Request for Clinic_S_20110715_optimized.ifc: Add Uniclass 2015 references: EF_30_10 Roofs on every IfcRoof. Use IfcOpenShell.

First a look at what the model holds.

```python
import ifcopenshell

model = ifcopenshell.open("Clinic_S_20110715_optimized.ifc")
print(model.schema)
print("classifications:", [c.Name for c in model.by_type("IfcClassification")])
for ifc_class in ("IfcDoor", "IfcRoof", "IfcStair", "IfcWall", "IfcWindow"):
    print(ifc_class, len(model.by_type(ifc_class)))
```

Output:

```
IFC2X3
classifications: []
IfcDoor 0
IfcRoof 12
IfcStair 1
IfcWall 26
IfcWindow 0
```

```python
import ifcopenshell
import ifcopenshell.api.classification

model = ifcopenshell.open("Clinic_S_20110715_optimized.ifc")

# IFC2X3 requires Source and Edition and has no link from the project to the system.
system = model.create_entity("IfcClassification", Source="NBS", Edition="2015", Name="Uniclass 2015")

codes = {
    "IfcRoof": ("EF_30_10", "Roofs"),
}
for ifc_class, (code, name) in codes.items():
    products = model.by_type(ifc_class)
    ifcopenshell.api.classification.add_reference(
        model, products=products, classification=system, identification=code, name=name
    )
    print(code, len(products))

model.write("Clinic_S_20110715_optimized_edited.ifc")
```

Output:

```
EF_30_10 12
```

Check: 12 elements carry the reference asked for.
